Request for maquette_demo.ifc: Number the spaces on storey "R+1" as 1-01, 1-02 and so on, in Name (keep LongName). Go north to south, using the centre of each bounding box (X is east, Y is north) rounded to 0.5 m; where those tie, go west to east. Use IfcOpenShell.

First a look at what the model holds.

```python
import ifcopenshell
import ifcopenshell.util.element
import ifcopenshell.util.placement

model = ifcopenshell.open("maquette_demo.ifc")
print(model.schema)
storey = next(s for s in model.by_type("IfcBuildingStorey") if s.Name == "R+1")
spaces = [e for e in ifcopenshell.util.element.get_decomposition(storey) if e.is_a("IfcSpace")]
for e in sorted(spaces, key=lambda e: e.id()):
    origin = ifcopenshell.util.placement.get_local_placement(e.ObjectPlacement)[:3, 3]
    print(e.id(), e.Name, e.LongName, origin.round(2) + 0.0, sep=" | ")
```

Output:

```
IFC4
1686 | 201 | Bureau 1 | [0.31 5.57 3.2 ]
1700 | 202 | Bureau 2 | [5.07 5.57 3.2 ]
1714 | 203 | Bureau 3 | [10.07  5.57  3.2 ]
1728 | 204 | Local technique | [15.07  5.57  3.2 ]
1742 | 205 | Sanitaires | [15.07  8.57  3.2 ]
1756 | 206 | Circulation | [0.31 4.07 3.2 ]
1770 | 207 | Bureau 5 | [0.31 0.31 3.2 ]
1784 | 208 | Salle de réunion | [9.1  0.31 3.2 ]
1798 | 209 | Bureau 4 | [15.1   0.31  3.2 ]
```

```python
import ifcopenshell
import ifcopenshell.geom
import ifcopenshell.util.element
import ifcopenshell.util.shape

model = ifcopenshell.open("maquette_demo.ifc")
settings = ifcopenshell.geom.settings()
settings.set("use-world-coords", True)


def centre(element):
    shape = ifcopenshell.geom.create_shape(settings, element)
    return ifcopenshell.util.shape.get_bbox_centroid(shape.geometry)


storey = next(s for s in model.by_type("IfcBuildingStorey") if s.Name == "R+1")
spaces = [e for e in ifcopenshell.util.element.get_decomposition(storey) if e.is_a("IfcSpace")]

# Insertion points can sit at a corner or the storey origin, so sort by the geometry (in metres).
centres = {e: centre(e) for e in spaces}
spaces.sort(key=lambda e: (-round(centres[e][1] / 0.5), centres[e][0]))

for i, e in enumerate(spaces, start=1):
    number = f"1-{i:02d}"
    e.Name = number
    print(e.id(), number)

model.write("maquette_demo_v2.ifc")
```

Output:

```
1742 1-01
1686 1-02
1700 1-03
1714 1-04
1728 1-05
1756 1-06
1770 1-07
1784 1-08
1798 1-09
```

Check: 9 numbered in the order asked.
